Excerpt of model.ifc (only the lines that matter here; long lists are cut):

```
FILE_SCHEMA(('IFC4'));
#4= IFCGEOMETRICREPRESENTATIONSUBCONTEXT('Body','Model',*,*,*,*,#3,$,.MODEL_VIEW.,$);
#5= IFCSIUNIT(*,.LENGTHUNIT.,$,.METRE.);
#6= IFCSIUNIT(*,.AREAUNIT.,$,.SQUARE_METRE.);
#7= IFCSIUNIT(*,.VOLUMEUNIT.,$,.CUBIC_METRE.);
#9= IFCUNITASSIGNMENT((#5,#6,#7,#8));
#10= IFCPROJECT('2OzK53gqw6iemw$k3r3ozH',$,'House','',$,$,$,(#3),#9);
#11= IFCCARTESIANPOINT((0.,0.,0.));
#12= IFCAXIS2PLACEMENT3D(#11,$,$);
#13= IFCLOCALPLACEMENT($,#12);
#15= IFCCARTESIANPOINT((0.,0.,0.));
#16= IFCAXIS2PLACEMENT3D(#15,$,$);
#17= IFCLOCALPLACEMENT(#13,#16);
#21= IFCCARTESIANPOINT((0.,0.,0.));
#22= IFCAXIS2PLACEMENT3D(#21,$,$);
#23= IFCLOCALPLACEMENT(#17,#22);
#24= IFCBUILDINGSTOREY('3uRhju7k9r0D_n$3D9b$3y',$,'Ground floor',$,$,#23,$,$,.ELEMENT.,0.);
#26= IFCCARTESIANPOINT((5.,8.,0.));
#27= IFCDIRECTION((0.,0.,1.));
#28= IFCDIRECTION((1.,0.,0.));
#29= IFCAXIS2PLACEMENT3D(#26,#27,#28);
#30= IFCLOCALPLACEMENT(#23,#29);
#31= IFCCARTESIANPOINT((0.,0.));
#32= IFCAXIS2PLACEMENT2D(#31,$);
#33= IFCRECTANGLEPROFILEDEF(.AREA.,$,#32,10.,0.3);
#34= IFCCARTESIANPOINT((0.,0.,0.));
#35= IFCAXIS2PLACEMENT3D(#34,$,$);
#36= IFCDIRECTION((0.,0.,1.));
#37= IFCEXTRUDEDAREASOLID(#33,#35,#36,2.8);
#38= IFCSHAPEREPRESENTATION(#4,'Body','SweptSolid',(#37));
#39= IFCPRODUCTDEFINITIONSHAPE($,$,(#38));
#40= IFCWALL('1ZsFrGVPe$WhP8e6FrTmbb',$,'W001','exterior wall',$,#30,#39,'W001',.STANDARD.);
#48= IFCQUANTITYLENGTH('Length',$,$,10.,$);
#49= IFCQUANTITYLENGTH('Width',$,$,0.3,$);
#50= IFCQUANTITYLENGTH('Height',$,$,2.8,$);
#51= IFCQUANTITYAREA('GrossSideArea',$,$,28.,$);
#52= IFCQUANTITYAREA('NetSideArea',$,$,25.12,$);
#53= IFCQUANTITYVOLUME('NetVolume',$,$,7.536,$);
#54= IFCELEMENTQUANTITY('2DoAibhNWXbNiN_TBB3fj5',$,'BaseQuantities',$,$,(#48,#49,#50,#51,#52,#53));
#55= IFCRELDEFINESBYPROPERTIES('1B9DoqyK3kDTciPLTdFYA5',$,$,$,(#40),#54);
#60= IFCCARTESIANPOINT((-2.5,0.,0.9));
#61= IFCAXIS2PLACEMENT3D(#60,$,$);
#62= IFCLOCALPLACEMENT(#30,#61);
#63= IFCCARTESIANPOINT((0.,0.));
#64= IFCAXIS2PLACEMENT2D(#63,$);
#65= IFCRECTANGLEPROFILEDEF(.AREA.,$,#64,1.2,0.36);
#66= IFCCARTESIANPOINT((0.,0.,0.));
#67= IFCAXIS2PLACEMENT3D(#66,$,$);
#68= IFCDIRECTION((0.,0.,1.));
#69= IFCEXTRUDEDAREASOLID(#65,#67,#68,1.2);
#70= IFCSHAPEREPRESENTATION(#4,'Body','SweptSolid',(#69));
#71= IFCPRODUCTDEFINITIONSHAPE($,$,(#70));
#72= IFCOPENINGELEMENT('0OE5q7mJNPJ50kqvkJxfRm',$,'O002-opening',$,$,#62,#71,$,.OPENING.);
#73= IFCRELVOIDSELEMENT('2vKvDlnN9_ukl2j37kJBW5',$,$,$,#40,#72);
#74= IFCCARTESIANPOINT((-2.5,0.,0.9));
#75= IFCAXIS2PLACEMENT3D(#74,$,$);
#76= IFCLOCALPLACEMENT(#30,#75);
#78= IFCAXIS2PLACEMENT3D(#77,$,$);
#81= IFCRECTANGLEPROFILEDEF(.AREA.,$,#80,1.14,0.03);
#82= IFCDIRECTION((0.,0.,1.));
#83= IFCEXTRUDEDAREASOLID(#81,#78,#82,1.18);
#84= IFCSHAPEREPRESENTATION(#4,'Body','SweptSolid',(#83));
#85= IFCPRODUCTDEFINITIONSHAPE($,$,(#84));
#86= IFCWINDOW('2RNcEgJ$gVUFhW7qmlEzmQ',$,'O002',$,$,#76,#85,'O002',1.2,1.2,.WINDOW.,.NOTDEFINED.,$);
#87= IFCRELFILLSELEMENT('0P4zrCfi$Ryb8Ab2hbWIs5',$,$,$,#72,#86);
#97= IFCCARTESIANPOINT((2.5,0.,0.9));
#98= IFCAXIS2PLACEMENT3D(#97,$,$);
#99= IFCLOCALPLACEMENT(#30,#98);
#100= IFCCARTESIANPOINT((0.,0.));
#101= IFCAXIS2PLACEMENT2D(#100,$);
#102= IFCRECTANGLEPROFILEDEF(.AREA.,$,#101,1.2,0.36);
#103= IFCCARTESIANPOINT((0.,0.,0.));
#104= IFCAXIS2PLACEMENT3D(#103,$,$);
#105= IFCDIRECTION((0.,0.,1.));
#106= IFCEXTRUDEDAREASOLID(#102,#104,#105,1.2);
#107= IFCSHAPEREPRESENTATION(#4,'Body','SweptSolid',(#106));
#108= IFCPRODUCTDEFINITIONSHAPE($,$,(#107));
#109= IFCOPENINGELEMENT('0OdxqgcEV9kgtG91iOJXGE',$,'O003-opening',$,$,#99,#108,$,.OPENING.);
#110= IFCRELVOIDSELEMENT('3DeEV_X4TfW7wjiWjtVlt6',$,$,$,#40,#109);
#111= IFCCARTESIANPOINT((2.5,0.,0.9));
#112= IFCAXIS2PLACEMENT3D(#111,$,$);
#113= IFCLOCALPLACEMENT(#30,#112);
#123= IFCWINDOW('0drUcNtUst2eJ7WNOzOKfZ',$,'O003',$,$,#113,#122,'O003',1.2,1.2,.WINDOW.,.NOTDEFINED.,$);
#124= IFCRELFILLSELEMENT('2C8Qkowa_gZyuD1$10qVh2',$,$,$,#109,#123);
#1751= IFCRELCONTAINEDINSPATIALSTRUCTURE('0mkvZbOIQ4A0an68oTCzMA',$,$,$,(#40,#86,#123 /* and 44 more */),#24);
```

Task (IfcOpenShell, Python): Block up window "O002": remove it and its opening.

```python
import ifcopenshell
import ifcopenshell.api.feature
import ifcopenshell.api.pset
import ifcopenshell.api.root
import ifcopenshell.geom
import ifcopenshell.util.element
import ifcopenshell.util.shape
import ifcopenshell.util.unit

model = ifcopenshell.open("model.ifc")
area_scale = ifcopenshell.util.unit.calculate_unit_scale(model, "AREAUNIT")
volume_scale = ifcopenshell.util.unit.calculate_unit_scale(model, "VOLUMEUNIT")
settings = ifcopenshell.geom.settings()


def volume(element):
    """Net volume in cubic metres, openings subtracted."""
    shape = ifcopenshell.geom.create_shape(settings, element)
    return ifcopenshell.util.shape.get_volume(shape.geometry)


window = model.by_guid("2RNcEgJ$gVUFhW7qmlEzmQ")
opening = window.FillsVoids[0].RelatingOpeningElement
wall = opening.VoidsElements[0].RelatingBuildingElement
before = volume(wall)

ifcopenshell.api.root.remove_product(model, product=window)
ifcopenshell.api.feature.remove_feature(model, feature=opening)

after = volume(wall)
thickness = 0.3  # wall thickness in metres

# Update the wall's stored quantities.
qto = model.by_id(ifcopenshell.util.element.get_pset(wall, "BaseQuantities", should_inherit=False)["id"])
ifcopenshell.api.pset.edit_qto(model, qto=qto, properties={
    "NetSideArea": after / thickness / area_scale,
    "NetVolume": after / volume_scale,
})

print(f"wall volume {before:.3f} -> {after:.3f} m3")

model.write("model_rev.ifc")
```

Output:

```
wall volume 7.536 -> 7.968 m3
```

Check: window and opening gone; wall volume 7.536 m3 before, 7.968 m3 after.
